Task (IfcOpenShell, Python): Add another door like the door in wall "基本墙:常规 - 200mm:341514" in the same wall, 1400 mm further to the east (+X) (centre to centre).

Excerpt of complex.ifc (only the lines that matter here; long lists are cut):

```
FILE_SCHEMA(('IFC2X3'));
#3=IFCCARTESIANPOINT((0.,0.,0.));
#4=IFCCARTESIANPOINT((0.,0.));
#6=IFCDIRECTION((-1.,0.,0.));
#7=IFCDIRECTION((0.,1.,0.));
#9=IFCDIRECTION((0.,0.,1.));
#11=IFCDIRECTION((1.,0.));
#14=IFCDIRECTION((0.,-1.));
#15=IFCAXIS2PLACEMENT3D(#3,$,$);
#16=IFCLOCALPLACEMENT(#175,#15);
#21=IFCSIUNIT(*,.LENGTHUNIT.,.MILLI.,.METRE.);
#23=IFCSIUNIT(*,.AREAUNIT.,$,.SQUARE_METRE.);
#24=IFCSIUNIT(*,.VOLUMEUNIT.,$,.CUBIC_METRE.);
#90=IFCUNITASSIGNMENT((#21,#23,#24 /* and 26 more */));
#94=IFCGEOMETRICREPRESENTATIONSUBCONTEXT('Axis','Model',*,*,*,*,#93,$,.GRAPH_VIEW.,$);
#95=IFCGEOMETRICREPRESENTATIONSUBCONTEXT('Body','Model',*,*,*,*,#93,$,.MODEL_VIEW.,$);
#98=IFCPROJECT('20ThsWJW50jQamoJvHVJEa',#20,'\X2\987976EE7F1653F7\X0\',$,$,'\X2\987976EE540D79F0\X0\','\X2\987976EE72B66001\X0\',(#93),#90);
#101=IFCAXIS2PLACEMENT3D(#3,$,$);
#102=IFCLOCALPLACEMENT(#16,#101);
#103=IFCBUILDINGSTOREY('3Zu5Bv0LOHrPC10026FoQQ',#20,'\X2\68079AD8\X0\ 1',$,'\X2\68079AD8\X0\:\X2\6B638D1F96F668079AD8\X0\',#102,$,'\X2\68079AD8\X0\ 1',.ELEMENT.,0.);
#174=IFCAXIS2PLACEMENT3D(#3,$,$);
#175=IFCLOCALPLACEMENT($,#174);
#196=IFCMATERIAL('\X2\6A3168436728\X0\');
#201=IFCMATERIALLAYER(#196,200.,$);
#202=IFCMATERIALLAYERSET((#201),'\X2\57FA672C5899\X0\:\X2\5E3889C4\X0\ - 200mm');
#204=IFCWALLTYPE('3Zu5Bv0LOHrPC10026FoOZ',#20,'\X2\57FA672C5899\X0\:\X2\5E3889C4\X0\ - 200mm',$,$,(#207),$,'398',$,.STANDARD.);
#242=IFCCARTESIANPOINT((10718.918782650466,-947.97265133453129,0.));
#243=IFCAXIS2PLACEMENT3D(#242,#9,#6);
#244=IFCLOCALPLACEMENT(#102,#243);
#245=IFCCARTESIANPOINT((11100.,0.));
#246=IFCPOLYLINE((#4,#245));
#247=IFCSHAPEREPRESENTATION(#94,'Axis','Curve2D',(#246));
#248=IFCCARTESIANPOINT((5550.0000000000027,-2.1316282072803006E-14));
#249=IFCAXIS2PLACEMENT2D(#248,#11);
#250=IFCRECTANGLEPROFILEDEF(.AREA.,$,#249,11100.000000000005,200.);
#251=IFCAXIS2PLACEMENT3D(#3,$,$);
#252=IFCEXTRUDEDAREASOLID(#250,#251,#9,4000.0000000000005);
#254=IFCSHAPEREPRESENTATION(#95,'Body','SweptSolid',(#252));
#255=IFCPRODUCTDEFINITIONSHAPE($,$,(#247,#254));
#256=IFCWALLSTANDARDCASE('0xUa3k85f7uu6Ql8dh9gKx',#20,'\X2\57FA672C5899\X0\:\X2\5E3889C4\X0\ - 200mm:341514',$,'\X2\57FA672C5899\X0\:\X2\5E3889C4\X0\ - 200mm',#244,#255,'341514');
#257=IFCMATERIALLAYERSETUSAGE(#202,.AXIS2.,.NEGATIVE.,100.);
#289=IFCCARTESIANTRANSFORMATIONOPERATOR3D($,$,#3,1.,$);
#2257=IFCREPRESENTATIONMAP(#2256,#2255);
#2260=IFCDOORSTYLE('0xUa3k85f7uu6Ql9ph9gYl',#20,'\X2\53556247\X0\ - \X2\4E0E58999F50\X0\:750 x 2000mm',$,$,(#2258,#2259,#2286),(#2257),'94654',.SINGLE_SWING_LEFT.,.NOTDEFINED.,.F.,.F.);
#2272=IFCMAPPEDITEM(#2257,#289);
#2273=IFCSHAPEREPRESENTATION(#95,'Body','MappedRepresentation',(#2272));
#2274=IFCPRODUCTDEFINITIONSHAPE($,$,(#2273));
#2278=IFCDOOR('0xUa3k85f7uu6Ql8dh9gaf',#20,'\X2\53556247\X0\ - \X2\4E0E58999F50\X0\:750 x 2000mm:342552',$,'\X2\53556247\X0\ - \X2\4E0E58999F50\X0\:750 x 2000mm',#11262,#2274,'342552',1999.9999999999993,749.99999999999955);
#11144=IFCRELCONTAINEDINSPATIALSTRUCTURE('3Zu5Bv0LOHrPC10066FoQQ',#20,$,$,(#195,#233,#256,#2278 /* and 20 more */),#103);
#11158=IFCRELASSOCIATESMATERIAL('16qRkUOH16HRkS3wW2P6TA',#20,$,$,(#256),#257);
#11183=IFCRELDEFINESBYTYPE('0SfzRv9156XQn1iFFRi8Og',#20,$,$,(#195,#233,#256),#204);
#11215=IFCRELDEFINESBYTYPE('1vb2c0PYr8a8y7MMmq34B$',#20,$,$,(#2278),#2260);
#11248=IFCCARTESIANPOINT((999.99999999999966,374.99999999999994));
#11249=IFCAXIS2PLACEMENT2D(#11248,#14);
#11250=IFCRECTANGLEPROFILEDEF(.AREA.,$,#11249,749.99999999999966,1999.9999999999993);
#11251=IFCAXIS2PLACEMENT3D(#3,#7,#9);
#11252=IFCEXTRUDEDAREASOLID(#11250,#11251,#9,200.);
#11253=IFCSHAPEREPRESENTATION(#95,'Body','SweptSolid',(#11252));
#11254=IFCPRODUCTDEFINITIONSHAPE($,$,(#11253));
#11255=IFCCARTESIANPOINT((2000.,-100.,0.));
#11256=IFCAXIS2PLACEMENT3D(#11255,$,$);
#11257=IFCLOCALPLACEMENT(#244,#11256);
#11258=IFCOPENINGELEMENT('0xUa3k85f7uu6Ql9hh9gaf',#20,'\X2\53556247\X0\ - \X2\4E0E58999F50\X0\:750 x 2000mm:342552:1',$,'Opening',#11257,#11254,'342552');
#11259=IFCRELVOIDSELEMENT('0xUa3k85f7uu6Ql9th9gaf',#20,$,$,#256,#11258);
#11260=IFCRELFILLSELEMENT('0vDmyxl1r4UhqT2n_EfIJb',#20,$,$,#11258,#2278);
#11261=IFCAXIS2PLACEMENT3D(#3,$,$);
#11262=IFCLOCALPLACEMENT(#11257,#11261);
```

```python
import ifcopenshell
import ifcopenshell.api.feature
import ifcopenshell.api.geometry
import ifcopenshell.api.root
import ifcopenshell.geom
import ifcopenshell.util.element
import ifcopenshell.util.placement
import ifcopenshell.util.shape
import ifcopenshell.util.unit

model = ifcopenshell.open("complex.ifc")
unit_scale = ifcopenshell.util.unit.calculate_unit_scale(model)
settings = ifcopenshell.geom.settings()


def volume(element):
    """Net volume in cubic metres, openings subtracted."""
    shape = ifcopenshell.geom.create_shape(settings, element)
    return ifcopenshell.util.shape.get_volume(shape.geometry)


def reuse_history(source, copy):
    """copy_class also copies each property set's owner history, people and application; keep the originals."""
    for rel in copy.IsDefinedBy:
        if rel.is_a("IfcRelDefinesByProperties") and (history := rel.RelatingPropertyDefinition.OwnerHistory):
            rel.RelatingPropertyDefinition.OwnerHistory = source.OwnerHistory
            ifcopenshell.util.element.remove_deep2(model, history)


door = model.by_guid("0xUa3k85f7uu6Ql8dh9gaf")
opening = door.FillsVoids[0].RelatingOpeningElement
wall = opening.VoidsElements[0].RelatingBuildingElement
before = volume(wall)
shift = ifcopenshell.util.placement.get_local_placement(wall.ObjectPlacement)[:3, 0] * -1.4 / unit_scale

# copy_class copies the void relationship, type, container and properties, but no geometry.
new_opening = ifcopenshell.api.root.copy_class(model, product=opening)
new_opening.Representation = ifcopenshell.util.element.copy_deep(
    model, opening.Representation, exclude=["IfcGeometricRepresentationContext", "IfcRepresentationMap"]
)
new_opening.Name = "单扇 - 与墙齐:750 x 2000mm"
new_opening.Tag = None
new_door = ifcopenshell.api.root.copy_class(model, product=door)
new_door.Representation = ifcopenshell.util.element.copy_deep(
    model, door.Representation, exclude=["IfcGeometricRepresentationContext", "IfcRepresentationMap"]
)
new_door.Name = "单扇 - 与墙齐:750 x 2000mm"
new_door.Tag = None
reuse_history(door, new_door)
fills = ifcopenshell.api.feature.add_filling(model, opening=new_opening, element=new_door)
fills.OwnerHistory = new_door.OwnerHistory  # required in IFC2X3

for old, new in ((opening, new_opening), (door, new_door)):
    matrix = ifcopenshell.util.placement.get_local_placement(old.ObjectPlacement)
    matrix[:3, 3] += shift
    ifcopenshell.api.geometry.edit_object_placement(model, product=new, matrix=matrix, is_si=False)

after = volume(wall)

print(f"wall volume {before:.3f} -> {after:.3f} m3")

model.write("complex_edited.ifc")
```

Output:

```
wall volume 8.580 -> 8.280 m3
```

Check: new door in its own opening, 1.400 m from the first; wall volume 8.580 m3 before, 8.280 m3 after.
